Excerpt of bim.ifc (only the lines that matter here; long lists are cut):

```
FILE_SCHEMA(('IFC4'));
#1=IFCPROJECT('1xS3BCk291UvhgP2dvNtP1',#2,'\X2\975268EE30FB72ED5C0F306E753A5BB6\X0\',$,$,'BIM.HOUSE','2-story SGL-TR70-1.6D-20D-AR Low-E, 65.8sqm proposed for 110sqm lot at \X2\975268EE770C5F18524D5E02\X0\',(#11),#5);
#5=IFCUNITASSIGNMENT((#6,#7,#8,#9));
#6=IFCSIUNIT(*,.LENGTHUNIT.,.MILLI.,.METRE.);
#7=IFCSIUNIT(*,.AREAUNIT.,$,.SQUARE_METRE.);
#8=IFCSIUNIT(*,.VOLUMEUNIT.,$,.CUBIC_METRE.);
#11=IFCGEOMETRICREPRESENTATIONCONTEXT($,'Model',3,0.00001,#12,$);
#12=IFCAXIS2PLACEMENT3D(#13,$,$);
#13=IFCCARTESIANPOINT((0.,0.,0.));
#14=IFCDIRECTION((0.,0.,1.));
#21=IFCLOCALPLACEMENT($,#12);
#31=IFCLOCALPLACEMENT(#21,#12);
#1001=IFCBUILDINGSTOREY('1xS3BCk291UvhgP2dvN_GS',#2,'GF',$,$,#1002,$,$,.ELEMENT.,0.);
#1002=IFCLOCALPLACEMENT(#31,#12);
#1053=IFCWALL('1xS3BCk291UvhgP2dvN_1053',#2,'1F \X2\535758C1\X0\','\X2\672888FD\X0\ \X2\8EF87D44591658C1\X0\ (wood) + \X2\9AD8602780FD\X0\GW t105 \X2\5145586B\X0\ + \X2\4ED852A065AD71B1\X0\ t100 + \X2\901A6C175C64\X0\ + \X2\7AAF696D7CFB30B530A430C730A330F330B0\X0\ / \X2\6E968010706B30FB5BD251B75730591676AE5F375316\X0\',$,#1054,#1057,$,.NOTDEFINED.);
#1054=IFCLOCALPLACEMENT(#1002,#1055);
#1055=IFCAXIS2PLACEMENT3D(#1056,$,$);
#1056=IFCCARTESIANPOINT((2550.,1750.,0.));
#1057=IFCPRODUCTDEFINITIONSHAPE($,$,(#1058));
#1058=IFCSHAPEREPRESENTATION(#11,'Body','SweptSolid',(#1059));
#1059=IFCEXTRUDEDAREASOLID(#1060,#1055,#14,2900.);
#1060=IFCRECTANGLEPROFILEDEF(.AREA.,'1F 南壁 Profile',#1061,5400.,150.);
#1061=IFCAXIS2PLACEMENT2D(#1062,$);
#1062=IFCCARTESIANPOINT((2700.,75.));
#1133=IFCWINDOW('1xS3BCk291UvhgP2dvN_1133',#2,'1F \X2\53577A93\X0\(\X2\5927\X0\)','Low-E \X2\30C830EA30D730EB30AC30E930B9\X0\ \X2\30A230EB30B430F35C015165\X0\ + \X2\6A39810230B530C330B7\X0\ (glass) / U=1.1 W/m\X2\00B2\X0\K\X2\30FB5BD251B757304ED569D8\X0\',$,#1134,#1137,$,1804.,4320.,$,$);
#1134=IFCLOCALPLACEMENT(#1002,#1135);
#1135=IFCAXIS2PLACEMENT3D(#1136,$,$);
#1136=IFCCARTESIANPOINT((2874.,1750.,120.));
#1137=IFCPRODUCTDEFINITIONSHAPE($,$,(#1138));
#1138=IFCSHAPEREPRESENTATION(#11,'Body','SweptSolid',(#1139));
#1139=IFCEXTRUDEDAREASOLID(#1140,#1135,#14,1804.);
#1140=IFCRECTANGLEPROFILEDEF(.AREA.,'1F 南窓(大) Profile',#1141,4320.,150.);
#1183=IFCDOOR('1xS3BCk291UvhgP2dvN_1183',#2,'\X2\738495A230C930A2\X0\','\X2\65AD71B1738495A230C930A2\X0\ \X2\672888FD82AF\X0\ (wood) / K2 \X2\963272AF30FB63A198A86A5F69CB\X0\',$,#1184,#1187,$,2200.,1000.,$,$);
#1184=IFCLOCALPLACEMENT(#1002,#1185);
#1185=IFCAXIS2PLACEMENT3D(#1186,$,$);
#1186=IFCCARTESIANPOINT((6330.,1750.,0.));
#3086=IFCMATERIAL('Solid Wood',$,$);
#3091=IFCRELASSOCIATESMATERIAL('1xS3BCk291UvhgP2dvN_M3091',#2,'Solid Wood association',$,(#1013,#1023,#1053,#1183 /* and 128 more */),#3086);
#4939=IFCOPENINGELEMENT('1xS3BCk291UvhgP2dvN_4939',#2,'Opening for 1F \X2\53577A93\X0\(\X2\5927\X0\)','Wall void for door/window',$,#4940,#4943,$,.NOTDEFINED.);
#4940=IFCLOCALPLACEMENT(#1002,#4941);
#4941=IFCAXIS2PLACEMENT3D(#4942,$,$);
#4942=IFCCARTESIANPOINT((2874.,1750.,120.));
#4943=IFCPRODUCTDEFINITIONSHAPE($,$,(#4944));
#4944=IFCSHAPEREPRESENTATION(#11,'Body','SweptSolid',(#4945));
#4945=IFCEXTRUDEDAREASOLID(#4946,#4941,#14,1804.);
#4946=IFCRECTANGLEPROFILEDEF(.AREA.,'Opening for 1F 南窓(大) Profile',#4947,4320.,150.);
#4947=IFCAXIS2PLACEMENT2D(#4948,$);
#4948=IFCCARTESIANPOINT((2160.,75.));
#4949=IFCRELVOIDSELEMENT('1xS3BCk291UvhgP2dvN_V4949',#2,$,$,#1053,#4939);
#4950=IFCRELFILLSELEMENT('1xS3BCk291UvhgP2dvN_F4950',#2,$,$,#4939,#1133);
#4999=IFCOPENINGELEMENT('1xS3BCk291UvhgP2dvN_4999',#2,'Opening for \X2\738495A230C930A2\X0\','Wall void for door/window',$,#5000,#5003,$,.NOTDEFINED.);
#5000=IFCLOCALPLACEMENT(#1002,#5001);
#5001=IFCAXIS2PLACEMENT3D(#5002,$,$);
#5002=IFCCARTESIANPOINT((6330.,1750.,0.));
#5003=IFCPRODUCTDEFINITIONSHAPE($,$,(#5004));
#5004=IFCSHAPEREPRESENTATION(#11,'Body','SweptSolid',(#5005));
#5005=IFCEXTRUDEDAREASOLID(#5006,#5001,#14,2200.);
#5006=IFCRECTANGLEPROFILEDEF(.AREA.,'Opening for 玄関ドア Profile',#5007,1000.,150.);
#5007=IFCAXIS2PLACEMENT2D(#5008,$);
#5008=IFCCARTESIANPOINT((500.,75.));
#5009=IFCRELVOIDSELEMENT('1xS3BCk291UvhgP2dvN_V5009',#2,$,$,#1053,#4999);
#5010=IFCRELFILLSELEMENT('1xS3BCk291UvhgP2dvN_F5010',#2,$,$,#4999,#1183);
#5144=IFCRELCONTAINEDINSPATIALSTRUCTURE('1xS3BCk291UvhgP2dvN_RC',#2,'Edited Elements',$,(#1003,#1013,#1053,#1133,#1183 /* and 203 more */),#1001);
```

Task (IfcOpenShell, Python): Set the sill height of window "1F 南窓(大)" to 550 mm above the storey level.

```python
import numpy as np
import ifcopenshell
import ifcopenshell.api.geometry
import ifcopenshell.geom
import ifcopenshell.util.element
import ifcopenshell.util.placement
import ifcopenshell.util.shape
import ifcopenshell.util.unit

model = ifcopenshell.open("bim.ifc")
unit_scale = ifcopenshell.util.unit.calculate_unit_scale(model)

window = model.by_id(1133)
opening = window.FillsVoids[0].RelatingOpeningElement
storey = ifcopenshell.util.element.get_container(window, ifc_class="IfcBuildingStorey")
level = ifcopenshell.util.placement.get_local_placement(storey.ObjectPlacement)[2, 3]

# The opening's origin need not be at the sill, so measure its lowest point.
shape = ifcopenshell.geom.create_shape(ifcopenshell.geom.settings(), opening)
bottom = ifcopenshell.util.shape.get_shape_bottom_elevation(shape, shape.geometry) / unit_scale
dz = level + 550.0 - bottom

shift = np.array([0.0, 0.0, dz])
# The window is not placed relative to its opening, so move both.
for product in (opening, window):
    matrix = ifcopenshell.util.placement.get_local_placement(product.ObjectPlacement)
    matrix[:3, 3] += shift
    ifcopenshell.api.geometry.edit_object_placement(model, product=product, matrix=matrix, is_si=False)

print(f"moved by {dz * unit_scale:+.3f} m")

model.write("bim_v2.ifc")
```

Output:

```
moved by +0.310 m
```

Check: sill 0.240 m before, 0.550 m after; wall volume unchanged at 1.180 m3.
